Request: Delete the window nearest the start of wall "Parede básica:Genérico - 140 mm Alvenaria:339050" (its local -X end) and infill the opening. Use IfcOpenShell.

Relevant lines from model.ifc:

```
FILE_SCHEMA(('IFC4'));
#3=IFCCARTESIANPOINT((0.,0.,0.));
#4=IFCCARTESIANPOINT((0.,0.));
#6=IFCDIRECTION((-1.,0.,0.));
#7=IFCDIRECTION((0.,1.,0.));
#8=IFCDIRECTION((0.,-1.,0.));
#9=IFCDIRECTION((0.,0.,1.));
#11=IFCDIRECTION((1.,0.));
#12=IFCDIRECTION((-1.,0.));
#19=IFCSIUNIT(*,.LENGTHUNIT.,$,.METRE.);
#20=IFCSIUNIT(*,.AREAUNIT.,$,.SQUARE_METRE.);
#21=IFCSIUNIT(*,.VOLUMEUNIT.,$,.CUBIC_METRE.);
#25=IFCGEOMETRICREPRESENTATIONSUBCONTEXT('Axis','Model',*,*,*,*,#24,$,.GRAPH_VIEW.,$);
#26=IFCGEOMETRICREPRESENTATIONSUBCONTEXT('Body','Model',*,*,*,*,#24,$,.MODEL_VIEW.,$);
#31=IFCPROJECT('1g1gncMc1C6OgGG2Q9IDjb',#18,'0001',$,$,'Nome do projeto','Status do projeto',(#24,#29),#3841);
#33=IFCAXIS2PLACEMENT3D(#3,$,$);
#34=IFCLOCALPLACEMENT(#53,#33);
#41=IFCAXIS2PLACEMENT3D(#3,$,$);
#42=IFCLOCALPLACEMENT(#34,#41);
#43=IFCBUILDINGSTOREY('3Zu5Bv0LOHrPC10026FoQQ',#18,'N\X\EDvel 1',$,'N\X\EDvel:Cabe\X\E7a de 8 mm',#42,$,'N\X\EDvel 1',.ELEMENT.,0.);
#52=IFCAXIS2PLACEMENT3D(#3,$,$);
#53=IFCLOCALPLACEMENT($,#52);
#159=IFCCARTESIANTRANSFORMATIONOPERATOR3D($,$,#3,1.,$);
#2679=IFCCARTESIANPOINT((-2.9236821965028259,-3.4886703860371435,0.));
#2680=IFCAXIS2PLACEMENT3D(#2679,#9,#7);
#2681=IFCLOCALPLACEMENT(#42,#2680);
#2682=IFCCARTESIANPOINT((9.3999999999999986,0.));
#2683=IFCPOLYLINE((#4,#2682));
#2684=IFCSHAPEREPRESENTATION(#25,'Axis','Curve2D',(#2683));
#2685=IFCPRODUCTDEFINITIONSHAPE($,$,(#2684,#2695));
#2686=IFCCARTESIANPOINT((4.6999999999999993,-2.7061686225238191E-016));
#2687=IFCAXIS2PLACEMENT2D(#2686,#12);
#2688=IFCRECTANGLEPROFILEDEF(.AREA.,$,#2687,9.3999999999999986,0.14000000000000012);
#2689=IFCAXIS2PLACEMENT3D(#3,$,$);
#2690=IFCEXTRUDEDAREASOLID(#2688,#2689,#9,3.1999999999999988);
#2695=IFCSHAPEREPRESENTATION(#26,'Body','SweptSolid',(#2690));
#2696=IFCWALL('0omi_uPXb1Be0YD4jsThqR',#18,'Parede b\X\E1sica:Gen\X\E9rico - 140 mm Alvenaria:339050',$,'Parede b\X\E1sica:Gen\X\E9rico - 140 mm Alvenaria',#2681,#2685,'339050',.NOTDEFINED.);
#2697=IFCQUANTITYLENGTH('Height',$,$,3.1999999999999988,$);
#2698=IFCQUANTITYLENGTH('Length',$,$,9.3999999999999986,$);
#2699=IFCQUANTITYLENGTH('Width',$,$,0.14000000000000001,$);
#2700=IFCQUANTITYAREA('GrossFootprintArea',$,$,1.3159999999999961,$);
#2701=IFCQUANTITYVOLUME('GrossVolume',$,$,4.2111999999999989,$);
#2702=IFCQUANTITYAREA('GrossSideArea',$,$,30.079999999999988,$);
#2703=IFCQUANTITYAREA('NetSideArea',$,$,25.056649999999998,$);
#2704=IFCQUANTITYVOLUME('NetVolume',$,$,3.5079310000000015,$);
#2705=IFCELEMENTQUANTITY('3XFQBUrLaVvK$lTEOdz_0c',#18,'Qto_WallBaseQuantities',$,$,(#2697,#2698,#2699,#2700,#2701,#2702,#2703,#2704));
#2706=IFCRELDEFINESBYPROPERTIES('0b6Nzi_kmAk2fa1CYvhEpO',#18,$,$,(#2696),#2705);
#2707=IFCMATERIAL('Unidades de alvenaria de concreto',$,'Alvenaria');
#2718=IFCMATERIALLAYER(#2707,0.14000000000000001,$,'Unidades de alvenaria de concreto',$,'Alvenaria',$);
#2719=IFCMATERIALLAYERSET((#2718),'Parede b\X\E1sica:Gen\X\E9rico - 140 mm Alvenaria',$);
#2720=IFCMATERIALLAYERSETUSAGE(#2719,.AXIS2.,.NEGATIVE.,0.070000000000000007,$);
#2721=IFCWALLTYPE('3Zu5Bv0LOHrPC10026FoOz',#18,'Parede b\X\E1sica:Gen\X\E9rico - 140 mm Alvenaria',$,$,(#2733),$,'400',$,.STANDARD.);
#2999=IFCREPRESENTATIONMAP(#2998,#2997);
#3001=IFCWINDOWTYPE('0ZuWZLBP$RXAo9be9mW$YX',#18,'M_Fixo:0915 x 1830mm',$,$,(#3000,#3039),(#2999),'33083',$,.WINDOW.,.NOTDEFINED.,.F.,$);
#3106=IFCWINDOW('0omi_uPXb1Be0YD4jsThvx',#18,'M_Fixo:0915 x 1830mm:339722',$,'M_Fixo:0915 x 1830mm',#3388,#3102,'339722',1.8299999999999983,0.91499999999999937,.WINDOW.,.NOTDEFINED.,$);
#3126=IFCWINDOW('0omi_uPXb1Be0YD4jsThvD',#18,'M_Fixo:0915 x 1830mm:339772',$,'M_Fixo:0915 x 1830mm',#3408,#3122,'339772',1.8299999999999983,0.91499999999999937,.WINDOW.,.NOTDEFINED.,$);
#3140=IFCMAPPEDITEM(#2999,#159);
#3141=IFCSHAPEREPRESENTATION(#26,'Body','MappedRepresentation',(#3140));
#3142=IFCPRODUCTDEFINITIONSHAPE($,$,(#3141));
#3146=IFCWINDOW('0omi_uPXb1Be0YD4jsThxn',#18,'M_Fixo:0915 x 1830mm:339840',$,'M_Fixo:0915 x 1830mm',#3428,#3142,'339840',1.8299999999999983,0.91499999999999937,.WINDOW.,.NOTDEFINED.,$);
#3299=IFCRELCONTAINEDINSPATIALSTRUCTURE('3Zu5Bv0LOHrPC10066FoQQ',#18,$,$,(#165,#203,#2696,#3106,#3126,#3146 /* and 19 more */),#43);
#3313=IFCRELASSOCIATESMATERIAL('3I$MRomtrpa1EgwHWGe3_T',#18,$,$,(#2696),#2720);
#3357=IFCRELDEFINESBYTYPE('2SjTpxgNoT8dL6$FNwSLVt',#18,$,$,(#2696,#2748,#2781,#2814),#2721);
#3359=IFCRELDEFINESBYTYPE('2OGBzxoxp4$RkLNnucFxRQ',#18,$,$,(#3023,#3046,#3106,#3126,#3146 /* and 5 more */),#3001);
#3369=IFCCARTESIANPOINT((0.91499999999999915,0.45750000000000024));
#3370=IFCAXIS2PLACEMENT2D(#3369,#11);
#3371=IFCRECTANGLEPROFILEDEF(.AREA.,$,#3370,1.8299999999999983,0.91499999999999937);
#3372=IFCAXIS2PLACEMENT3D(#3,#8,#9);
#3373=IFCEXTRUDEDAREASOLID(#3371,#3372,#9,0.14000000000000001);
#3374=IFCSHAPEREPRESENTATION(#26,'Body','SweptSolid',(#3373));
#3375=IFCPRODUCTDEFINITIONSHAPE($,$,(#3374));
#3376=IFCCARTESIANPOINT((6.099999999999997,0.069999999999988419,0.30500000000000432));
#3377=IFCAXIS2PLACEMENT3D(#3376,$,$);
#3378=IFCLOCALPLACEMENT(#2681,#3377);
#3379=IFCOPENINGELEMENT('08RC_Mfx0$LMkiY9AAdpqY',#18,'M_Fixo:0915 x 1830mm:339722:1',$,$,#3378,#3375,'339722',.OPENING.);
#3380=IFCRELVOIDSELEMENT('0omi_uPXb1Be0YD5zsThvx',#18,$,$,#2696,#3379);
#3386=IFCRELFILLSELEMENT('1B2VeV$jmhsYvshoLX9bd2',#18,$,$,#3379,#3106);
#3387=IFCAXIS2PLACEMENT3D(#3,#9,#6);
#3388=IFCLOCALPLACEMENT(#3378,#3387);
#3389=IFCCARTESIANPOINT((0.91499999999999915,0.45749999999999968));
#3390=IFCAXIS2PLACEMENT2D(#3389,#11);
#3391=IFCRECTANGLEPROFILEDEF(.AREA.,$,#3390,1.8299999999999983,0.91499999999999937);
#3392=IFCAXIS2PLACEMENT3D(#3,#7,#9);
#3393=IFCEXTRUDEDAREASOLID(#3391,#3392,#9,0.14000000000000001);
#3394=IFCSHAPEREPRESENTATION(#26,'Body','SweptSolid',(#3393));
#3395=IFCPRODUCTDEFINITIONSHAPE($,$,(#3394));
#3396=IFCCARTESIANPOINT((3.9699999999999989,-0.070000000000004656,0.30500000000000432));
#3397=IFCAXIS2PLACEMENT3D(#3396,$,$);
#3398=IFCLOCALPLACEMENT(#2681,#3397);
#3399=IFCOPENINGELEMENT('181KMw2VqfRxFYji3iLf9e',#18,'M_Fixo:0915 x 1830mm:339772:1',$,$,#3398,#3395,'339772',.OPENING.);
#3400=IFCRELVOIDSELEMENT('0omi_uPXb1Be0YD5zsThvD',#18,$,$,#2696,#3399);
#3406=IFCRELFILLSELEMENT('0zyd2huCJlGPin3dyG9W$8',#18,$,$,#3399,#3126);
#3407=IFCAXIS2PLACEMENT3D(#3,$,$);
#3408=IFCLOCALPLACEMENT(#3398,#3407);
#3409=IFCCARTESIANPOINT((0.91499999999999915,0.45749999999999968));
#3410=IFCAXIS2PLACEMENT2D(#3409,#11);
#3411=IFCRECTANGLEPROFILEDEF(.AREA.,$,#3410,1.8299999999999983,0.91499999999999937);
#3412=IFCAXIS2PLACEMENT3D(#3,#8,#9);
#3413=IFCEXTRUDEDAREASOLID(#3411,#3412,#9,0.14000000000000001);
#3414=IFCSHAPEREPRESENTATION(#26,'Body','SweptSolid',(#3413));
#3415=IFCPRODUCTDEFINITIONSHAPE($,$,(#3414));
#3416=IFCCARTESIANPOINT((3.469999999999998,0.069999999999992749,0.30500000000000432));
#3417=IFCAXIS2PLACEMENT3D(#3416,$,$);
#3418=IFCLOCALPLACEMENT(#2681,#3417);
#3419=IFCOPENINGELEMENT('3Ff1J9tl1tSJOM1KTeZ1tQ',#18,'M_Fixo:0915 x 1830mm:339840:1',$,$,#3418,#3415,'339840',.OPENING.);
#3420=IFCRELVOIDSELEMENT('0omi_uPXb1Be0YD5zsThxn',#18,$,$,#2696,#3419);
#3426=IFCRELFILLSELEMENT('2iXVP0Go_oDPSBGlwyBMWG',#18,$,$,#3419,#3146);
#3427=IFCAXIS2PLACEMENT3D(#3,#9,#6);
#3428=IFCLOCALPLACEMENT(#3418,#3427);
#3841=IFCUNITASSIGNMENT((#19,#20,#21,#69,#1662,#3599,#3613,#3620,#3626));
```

```python
import ifcopenshell
import ifcopenshell.api.feature
import ifcopenshell.api.pset
import ifcopenshell.api.root
import ifcopenshell.geom
import ifcopenshell.util.element
import ifcopenshell.util.shape
import ifcopenshell.util.unit

model = ifcopenshell.open("model.ifc")
area_scale = ifcopenshell.util.unit.calculate_unit_scale(model, "AREAUNIT")
volume_scale = ifcopenshell.util.unit.calculate_unit_scale(model, "VOLUMEUNIT")
settings = ifcopenshell.geom.settings()


def volume(element):
    """Net volume in cubic metres, openings subtracted."""
    shape = ifcopenshell.geom.create_shape(settings, element)
    return ifcopenshell.util.shape.get_volume(shape.geometry)


window = model.by_id(3146)
opening = window.FillsVoids[0].RelatingOpeningElement
wall = opening.VoidsElements[0].RelatingBuildingElement
before = volume(wall)

ifcopenshell.api.root.remove_product(model, product=window)
ifcopenshell.api.feature.remove_feature(model, feature=opening)

after = volume(wall)
thickness = 0.14  # wall thickness in metres

# Update the wall's stored quantities.
qto = model.by_id(ifcopenshell.util.element.get_pset(wall, "Qto_WallBaseQuantities", should_inherit=False)["id"])
ifcopenshell.api.pset.edit_qto(model, qto=qto, properties={
    "NetSideArea": after / thickness / area_scale,
    "NetVolume": after / volume_scale,
})

print(f"wall volume {before:.3f} -> {after:.3f} m3")

model.write("model_rev.ifc")
```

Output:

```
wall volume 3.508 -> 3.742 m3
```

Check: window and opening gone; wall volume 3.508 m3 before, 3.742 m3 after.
